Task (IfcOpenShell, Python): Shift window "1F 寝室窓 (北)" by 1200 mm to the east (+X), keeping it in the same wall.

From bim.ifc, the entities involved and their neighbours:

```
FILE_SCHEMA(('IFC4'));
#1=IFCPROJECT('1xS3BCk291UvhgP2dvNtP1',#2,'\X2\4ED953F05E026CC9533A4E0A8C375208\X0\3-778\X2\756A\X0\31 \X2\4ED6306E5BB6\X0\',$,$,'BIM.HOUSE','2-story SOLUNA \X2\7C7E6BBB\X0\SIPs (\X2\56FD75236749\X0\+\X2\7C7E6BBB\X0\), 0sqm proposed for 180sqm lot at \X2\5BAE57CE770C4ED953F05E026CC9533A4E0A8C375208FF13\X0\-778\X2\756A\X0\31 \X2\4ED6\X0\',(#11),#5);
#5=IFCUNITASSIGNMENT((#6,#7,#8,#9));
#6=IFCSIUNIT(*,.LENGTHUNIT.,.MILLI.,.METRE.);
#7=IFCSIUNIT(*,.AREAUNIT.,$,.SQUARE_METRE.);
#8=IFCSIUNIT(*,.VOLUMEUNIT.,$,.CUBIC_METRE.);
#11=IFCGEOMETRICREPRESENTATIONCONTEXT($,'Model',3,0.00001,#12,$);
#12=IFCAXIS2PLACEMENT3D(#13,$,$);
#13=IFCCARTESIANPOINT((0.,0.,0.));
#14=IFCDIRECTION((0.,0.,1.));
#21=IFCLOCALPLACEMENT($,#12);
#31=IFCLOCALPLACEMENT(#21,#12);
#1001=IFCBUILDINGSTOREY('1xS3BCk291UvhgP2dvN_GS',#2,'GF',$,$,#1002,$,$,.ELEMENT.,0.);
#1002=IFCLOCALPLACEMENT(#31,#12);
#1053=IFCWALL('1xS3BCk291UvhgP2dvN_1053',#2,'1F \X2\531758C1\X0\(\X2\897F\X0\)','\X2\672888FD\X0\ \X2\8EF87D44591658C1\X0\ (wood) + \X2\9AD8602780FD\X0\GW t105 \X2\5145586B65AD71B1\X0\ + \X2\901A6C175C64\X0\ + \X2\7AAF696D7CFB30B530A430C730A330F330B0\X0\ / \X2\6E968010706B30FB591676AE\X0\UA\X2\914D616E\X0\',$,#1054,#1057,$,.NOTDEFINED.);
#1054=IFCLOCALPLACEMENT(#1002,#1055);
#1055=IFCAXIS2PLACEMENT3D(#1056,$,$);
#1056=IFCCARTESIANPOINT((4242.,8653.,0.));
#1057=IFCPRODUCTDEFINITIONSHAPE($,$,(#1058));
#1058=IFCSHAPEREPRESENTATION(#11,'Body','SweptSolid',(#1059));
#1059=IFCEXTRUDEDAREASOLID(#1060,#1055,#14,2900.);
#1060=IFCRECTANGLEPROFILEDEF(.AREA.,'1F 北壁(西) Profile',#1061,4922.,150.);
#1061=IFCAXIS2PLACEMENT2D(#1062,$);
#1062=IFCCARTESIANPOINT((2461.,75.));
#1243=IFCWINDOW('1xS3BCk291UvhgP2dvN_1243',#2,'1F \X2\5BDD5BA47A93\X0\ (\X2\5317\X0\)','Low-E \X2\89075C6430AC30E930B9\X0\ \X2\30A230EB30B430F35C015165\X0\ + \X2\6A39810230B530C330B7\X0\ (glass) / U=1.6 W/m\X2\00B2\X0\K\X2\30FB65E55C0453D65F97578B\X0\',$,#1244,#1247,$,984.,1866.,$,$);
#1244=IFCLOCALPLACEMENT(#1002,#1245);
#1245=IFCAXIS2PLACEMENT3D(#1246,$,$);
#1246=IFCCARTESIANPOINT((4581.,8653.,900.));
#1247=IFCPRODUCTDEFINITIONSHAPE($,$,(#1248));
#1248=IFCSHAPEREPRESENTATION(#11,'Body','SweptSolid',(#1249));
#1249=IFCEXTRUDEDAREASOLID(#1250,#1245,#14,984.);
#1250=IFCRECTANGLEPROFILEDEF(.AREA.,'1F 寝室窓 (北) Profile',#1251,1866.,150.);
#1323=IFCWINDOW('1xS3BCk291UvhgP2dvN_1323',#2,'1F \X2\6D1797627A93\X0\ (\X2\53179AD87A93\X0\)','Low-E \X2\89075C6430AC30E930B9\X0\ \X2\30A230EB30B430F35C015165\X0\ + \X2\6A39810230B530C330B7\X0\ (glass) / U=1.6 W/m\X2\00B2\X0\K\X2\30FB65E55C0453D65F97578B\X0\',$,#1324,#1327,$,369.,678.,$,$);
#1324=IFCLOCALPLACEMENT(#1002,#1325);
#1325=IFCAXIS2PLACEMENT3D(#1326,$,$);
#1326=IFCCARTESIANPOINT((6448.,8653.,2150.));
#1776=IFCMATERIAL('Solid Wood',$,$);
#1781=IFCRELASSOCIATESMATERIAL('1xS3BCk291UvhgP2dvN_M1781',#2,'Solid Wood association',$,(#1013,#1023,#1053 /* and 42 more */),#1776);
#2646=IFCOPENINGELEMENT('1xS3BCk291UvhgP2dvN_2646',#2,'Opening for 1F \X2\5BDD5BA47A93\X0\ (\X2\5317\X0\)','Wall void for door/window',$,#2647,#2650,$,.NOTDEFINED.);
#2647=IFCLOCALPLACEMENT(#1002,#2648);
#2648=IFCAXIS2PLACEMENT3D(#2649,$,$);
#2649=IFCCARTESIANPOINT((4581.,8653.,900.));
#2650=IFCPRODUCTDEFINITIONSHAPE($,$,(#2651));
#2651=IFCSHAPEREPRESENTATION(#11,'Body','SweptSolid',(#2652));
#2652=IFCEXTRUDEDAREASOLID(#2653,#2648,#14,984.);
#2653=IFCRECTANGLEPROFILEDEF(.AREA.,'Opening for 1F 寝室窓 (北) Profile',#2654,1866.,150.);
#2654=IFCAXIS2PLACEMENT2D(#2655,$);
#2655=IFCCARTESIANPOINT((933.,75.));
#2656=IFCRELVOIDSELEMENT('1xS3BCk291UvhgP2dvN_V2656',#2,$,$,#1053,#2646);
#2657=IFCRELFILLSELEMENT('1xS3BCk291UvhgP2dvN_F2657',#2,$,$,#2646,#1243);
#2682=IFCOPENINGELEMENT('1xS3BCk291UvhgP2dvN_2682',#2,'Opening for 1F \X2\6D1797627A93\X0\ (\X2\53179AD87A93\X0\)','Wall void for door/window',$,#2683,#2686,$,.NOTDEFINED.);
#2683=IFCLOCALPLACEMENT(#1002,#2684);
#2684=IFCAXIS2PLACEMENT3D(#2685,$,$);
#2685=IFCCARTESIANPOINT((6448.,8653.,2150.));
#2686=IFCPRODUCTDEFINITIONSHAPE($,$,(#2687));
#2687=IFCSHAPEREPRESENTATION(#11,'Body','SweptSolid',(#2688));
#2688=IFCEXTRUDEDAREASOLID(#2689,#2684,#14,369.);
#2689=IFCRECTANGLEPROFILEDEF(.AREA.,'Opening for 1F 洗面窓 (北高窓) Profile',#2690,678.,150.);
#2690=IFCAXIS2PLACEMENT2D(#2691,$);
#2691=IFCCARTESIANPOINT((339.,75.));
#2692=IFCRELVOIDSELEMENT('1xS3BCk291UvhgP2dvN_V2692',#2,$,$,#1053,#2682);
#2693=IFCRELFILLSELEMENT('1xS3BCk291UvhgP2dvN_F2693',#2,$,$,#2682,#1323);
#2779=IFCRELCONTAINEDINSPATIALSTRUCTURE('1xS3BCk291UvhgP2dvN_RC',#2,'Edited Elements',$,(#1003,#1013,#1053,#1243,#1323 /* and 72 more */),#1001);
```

```python
import ifcopenshell
import ifcopenshell.api.geometry
import ifcopenshell.util.placement

model = ifcopenshell.open("bim.ifc")

window = model.by_guid("1xS3BCk291UvhgP2dvN_1243")
opening = window.FillsVoids[0].RelatingOpeningElement
wall = opening.VoidsElements[0].RelatingBuildingElement

wall_matrix = ifcopenshell.util.placement.get_local_placement(wall.ObjectPlacement)
shift = wall_matrix[:3, 0] * 1200.0
before = ifcopenshell.util.placement.get_local_placement(window.ObjectPlacement)[:3, 3].copy()

# The window is not placed relative to its opening, so move both.
for product in (opening, window):
    matrix = ifcopenshell.util.placement.get_local_placement(product.ObjectPlacement)
    matrix[:3, 3] += shift
    ifcopenshell.api.geometry.edit_object_placement(model, product=product, matrix=matrix, is_si=False)

after = ifcopenshell.util.placement.get_local_placement(window.ObjectPlacement)[:3, 3]
print("window moved by", (after - before).round(3) + 0.0)

model.write("bim_updated.ifc")
```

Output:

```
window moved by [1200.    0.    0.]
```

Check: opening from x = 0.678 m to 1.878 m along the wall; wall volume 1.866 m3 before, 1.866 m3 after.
